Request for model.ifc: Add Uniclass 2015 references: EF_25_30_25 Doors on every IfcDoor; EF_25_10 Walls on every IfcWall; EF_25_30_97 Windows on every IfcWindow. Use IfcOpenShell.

First a look at what the model holds.

```python
import ifcopenshell

model = ifcopenshell.open("model.ifc")
print(model.schema)
print("classifications:", [c.Name for c in model.by_type("IfcClassification")])
for ifc_class in ("IfcDoor", "IfcRoof", "IfcStair", "IfcWall", "IfcWindow"):
    print(ifc_class, len(model.by_type(ifc_class)))
```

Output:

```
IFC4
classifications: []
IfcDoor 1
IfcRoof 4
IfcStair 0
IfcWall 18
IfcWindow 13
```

```python
import ifcopenshell
import ifcopenshell.api.classification

model = ifcopenshell.open("model.ifc")

system = ifcopenshell.api.classification.add_classification(model, classification="Uniclass 2015")

codes = {
    "IfcDoor": ("EF_25_30_25", "Doors"),
    "IfcWall": ("EF_25_10", "Walls"),
    "IfcWindow": ("EF_25_30_97", "Windows"),
}
for ifc_class, (code, name) in codes.items():
    products = model.by_type(ifc_class)
    ifcopenshell.api.classification.add_reference(
        model, products=products, classification=system, identification=code, name=name
    )
    print(code, len(products))

model.write("model_updated.ifc")
```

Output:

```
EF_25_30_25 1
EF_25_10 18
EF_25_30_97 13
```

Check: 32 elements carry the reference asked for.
